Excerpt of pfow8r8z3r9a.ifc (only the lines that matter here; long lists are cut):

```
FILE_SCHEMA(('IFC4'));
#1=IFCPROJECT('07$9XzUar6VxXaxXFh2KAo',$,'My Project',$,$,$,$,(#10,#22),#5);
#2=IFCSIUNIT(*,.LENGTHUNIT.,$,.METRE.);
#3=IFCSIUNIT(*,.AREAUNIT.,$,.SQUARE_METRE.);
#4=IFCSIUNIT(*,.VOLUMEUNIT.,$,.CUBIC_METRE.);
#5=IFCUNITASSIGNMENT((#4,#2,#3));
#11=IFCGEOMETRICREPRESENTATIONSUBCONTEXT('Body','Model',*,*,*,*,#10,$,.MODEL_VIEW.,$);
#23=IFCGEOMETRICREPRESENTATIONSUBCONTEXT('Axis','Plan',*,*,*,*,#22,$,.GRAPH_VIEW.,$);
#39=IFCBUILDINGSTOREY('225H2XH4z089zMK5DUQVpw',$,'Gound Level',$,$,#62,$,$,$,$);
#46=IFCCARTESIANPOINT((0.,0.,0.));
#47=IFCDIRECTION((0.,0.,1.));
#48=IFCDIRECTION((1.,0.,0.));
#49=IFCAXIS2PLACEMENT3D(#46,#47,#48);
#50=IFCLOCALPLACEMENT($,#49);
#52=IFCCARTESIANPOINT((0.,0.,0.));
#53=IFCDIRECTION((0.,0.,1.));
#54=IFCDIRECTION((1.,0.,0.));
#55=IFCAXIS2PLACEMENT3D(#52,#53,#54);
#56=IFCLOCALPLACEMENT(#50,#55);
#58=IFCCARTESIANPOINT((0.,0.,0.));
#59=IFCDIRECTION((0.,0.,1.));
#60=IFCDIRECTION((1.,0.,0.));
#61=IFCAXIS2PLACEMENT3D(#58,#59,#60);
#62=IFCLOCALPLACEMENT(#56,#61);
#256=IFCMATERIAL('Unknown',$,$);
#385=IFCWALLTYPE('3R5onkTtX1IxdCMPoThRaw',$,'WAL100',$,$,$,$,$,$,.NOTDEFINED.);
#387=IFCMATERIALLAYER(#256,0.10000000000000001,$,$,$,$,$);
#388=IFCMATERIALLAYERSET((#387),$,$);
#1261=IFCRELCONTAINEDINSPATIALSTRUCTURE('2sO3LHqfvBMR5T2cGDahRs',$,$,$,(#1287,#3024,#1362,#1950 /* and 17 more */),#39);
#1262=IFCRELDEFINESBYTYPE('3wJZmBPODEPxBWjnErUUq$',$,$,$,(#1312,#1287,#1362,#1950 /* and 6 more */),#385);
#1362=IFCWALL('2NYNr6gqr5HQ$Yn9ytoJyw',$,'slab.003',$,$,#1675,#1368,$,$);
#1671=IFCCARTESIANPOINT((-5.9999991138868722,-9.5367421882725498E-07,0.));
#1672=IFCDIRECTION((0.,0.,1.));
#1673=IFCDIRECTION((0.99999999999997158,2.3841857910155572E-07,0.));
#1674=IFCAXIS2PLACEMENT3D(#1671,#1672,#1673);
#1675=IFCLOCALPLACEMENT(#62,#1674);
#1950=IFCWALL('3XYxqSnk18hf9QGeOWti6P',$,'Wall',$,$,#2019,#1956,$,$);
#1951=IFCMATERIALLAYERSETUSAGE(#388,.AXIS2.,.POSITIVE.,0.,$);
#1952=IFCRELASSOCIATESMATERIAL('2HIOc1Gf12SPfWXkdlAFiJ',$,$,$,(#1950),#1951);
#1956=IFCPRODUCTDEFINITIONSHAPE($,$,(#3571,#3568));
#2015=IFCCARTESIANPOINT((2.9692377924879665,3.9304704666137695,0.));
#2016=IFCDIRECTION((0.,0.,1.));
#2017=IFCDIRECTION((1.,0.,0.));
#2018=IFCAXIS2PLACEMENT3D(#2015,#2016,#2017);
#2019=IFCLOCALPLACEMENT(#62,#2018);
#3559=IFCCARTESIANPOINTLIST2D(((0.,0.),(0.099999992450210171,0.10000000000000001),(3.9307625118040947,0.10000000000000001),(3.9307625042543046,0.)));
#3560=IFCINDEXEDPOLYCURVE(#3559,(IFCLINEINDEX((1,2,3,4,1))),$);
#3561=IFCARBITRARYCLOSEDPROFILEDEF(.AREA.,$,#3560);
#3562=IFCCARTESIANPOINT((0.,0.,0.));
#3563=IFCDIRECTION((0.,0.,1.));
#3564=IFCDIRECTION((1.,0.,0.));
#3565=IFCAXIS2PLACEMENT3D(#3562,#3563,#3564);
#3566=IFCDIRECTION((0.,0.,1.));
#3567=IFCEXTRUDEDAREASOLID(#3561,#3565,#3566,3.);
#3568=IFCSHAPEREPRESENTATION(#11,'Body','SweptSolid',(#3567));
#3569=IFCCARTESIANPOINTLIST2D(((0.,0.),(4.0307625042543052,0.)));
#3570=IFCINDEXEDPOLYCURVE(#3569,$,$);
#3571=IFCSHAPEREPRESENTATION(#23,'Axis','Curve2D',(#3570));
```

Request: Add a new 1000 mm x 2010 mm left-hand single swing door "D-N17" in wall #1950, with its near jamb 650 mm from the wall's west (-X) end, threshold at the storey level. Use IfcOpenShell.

```python
import numpy as np
import ifcopenshell
import ifcopenshell.api.feature
import ifcopenshell.api.geometry
import ifcopenshell.api.root
import ifcopenshell.api.spatial
import ifcopenshell.geom
import ifcopenshell.util.element
import ifcopenshell.util.placement
import ifcopenshell.util.representation
import ifcopenshell.util.shape
import ifcopenshell.util.unit

model = ifcopenshell.open("pfow8r8z3r9a.ifc")
unit_scale = ifcopenshell.util.unit.calculate_unit_scale(model)
settings = ifcopenshell.geom.settings()


def volume(element):
    """Net volume in cubic metres, openings subtracted."""
    shape = ifcopenshell.geom.create_shape(settings, element)
    return ifcopenshell.util.shape.get_volume(shape.geometry)


wall = model.by_guid("3XYxqSnk18hf9QGeOWti6P")
storey = ifcopenshell.util.element.get_container(wall, ifc_class="IfcBuildingStorey")
context = ifcopenshell.util.representation.get_context(model, "Model", "Body", "MODEL_VIEW")
before = volume(wall)

width, height, from_end, sill = 1, 2.01, 0.65, 0.0  # metres

# The wall runs along its own X axis, and the end named is its -X end.
wall_shape = ifcopenshell.geom.create_shape(settings, wall)
x, y, z = ifcopenshell.util.shape.get_vertices(wall_shape.geometry).T
start = x.min() + from_end
face, thickness = float(y.min()), float(y.max() - y.min())
wall_matrix = ifcopenshell.util.placement.get_local_placement(wall.ObjectPlacement)
level = ifcopenshell.util.placement.get_local_placement(storey.ObjectPlacement)[2, 3]


def in_wall(x, y):
    """Placement at x, y metres in the wall's axes, at sill height."""
    matrix = wall_matrix.copy()
    matrix[:, 3] = wall_matrix @ np.array([x / unit_scale, y / unit_scale, 0.0, 1.0])
    matrix[2, 3] = level + sill / unit_scale
    return matrix


# Opening: a box that overshoots both wall faces by 50 mm.
opening = ifcopenshell.api.root.create_entity(model, ifc_class="IfcOpeningElement", predefined_type="OPENING")
box = ifcopenshell.api.geometry.add_wall_representation(
    model, context=context, length=width, height=height, thickness=thickness + 0.1
)
ifcopenshell.api.geometry.assign_representation(model, product=opening, representation=box)
ifcopenshell.api.geometry.edit_object_placement(model, product=opening, matrix=in_wall(start, face - 0.05), is_si=False)
ifcopenshell.api.feature.add_feature(model, feature=opening, element=wall)

door = ifcopenshell.api.root.create_entity(model, ifc_class="IfcDoor", name="D-N17", predefined_type="DOOR")
door.OverallWidth, door.OverallHeight = width / unit_scale, height / unit_scale
door.OperationType = "SINGLE_SWING_LEFT"
body = ifcopenshell.api.geometry.add_door_representation(
    model,
    context=context,
    overall_width=door.OverallWidth,
    overall_height=door.OverallHeight,
    operation_type="SINGLE_SWING_LEFT",
    lining_properties={"LiningDepth": thickness / unit_scale, "ThresholdDepth": thickness / unit_scale},
)
ifcopenshell.api.geometry.assign_representation(model, product=door, representation=body)
ifcopenshell.api.spatial.assign_container(model, products=[door], relating_structure=storey)
ifcopenshell.api.feature.add_filling(model, opening=opening, element=door)

# The lining spans the wall, so the door starts at the wall face.
ifcopenshell.api.geometry.edit_object_placement(model, product=door, matrix=in_wall(start, face), is_si=False)

after = volume(wall)

print(f"wall volume {before:.3f} -> {after:.3f} m3")

model.write("pfow8r8z3r9a-out.ifc")
```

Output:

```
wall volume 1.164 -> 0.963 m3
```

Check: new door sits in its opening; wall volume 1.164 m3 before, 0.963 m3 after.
